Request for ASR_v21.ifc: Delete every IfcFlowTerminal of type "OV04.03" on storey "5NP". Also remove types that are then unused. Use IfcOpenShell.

First a look at what the model holds.

```python
import ifcopenshell
import ifcopenshell.util.element

model = ifcopenshell.open("ASR_v21.ifc")
print(model.schema)
storey = next(s for s in model.by_type("IfcBuildingStorey") if s.Name == "5NP")
terminals = [e for e in ifcopenshell.util.element.get_decomposition(storey) if e.is_a("IfcFlowTerminal")]
seen = {}
for e in terminals:
    element_type = ifcopenshell.util.element.get_type(e)
    name = element_type.Name if element_type not in (None, e) else None
    seen[name] = seen.get(name, 0) + 1
for name, count in sorted(seen.items(), key=str):
    print(count, "x", name)
```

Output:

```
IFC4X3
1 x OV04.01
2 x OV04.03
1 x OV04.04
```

```python
import ifcopenshell
import ifcopenshell.api.root
import ifcopenshell.util.element

model = ifcopenshell.open("ASR_v21.ifc")

storey = next(s for s in model.by_type("IfcBuildingStorey") if s.Name == "5NP")
terminals = [e for e in ifcopenshell.util.element.get_decomposition(storey) if e.is_a("IfcFlowTerminal")]
targets = [e for e in terminals if (t := ifcopenshell.util.element.get_type(e)) not in (None, e) and t.Name == "OV04.03"]
types = {ifcopenshell.util.element.get_type(e) for e in targets} - {None, *targets}

for e in targets:
    ifcopenshell.api.root.remove_product(model, product=e)
print(len(targets), "removed")

unused = [t for t in types if not ifcopenshell.util.element.get_types(t)]
for t in unused:
    ifcopenshell.api.root.remove_product(model, product=t)
print(len(unused), "unused types removed")

model.write("ASR_v21_edited.ifc")
```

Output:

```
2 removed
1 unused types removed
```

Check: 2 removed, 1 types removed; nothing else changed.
